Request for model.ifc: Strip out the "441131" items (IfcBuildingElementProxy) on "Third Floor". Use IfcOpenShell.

First a look at what the model holds.

```python
import ifcopenshell
import ifcopenshell.util.element

model = ifcopenshell.open("model.ifc")
print(model.schema)
storey = next(s for s in model.by_type("IfcBuildingStorey") if s.Name == "Third Floor")
proxies = [e for e in ifcopenshell.util.element.get_decomposition(storey) if e.is_a("IfcBuildingElementProxy")]
seen = {}
for e in proxies:
    element_type = ifcopenshell.util.element.get_type(e)
    name = element_type.Name if element_type not in (None, e) else None
    seen[name] = seen.get(name, 0) + 1
for name, count in sorted(seen.items(), key=str):
    print(count, "x", name)
```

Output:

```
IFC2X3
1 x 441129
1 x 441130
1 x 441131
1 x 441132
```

```python
import ifcopenshell
import ifcopenshell.api.root
import ifcopenshell.util.element

model = ifcopenshell.open("model.ifc")

storey = next(s for s in model.by_type("IfcBuildingStorey") if s.Name == "Third Floor")
proxies = [e for e in ifcopenshell.util.element.get_decomposition(storey) if e.is_a("IfcBuildingElementProxy")]
targets = [e for e in proxies if (t := ifcopenshell.util.element.get_type(e)) not in (None, e) and t.Name == "441131"]

for e in targets:
    ifcopenshell.api.root.remove_product(model, product=e)
print(len(targets), "removed")

model.write("model_v2.ifc")
```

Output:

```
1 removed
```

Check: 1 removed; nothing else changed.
